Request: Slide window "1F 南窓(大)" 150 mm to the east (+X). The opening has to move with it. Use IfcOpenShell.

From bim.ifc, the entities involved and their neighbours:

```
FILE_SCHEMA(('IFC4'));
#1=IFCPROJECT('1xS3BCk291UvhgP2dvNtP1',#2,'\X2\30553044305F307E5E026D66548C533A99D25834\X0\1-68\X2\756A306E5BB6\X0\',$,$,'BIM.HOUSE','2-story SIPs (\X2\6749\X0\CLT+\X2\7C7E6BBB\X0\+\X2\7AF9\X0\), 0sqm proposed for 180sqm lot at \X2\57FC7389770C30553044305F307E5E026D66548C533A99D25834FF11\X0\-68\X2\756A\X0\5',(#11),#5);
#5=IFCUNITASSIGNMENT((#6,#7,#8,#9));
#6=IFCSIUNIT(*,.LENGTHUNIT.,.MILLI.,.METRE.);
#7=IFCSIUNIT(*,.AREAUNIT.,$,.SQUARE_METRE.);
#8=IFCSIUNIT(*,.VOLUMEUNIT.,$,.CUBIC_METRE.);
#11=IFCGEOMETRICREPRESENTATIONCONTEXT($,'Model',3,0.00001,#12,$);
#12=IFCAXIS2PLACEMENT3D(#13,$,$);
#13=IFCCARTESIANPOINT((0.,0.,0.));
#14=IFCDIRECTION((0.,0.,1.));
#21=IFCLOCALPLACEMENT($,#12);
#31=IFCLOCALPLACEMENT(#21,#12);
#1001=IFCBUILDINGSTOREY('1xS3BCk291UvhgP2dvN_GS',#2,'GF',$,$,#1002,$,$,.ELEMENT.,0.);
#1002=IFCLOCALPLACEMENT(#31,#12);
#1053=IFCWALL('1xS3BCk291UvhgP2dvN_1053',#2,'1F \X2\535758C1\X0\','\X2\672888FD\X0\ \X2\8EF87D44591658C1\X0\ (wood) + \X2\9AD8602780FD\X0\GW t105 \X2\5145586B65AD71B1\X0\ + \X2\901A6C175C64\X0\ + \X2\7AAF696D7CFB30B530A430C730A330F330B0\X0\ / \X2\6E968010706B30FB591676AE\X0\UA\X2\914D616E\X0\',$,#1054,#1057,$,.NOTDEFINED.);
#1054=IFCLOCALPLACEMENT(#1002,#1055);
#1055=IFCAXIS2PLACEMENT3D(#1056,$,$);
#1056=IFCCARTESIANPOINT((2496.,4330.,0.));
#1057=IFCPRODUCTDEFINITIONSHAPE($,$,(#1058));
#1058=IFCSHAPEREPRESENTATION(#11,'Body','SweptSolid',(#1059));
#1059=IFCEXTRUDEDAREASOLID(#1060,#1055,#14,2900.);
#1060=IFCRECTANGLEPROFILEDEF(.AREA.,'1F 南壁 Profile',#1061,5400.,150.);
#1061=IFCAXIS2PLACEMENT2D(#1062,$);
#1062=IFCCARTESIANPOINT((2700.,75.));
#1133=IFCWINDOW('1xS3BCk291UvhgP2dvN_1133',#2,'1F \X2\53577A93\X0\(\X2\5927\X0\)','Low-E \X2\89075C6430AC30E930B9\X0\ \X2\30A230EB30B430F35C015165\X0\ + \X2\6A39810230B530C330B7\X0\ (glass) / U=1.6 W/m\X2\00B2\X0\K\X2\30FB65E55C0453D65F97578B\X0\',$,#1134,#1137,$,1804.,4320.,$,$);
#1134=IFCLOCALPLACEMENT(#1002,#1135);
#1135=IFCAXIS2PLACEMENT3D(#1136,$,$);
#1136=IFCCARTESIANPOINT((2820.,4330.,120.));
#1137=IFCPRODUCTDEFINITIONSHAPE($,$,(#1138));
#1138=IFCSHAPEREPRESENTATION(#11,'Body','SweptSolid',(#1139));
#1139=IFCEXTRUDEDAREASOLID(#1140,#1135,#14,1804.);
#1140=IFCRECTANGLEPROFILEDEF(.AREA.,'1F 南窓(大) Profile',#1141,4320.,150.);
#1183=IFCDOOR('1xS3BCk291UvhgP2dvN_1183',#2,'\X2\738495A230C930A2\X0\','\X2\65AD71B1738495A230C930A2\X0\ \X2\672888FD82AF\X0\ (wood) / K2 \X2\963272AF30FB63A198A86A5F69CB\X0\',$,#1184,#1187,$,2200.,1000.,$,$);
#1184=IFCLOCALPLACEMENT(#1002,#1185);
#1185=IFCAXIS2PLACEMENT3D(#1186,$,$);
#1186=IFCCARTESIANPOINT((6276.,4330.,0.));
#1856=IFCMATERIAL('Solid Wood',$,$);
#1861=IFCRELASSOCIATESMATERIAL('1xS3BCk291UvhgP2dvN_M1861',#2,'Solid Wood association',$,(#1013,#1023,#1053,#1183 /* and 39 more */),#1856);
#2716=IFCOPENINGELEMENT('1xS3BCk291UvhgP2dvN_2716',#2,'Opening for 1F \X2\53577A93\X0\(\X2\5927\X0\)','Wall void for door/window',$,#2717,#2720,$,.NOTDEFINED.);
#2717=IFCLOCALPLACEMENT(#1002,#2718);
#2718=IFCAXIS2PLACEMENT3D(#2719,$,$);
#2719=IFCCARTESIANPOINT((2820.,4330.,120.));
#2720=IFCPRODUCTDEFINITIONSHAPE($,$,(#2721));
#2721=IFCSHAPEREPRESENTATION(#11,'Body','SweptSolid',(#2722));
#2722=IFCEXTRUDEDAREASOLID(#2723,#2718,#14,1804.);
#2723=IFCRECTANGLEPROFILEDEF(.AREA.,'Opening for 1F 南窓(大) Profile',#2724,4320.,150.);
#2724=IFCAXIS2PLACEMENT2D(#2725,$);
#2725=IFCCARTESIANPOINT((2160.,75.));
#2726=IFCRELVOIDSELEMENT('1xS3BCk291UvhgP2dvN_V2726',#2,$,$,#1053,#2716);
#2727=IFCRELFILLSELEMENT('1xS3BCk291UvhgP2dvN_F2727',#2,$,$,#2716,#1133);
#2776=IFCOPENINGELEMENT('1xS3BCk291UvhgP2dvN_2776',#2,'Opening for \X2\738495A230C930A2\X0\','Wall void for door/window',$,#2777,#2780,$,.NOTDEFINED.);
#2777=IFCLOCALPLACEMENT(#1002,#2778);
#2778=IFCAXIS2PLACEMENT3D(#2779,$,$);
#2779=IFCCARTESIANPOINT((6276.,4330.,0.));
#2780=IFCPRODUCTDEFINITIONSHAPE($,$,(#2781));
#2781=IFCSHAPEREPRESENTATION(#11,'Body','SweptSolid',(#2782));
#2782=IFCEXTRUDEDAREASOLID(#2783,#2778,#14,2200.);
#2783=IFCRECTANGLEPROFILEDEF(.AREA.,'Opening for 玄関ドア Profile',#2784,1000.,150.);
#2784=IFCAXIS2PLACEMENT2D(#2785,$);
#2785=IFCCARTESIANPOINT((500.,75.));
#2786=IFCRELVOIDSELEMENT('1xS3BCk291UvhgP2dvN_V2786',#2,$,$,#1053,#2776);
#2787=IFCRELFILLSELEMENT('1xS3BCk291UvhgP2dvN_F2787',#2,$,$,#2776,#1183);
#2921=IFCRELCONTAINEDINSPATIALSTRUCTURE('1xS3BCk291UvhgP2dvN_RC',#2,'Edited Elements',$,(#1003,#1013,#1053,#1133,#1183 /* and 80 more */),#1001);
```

```python
import ifcopenshell
import ifcopenshell.api.geometry
import ifcopenshell.util.placement
import ifcopenshell.util.unit

model = ifcopenshell.open("bim.ifc")
unit_scale = ifcopenshell.util.unit.calculate_unit_scale(model)

window = model.by_guid("1xS3BCk291UvhgP2dvN_1133")
opening = window.FillsVoids[0].RelatingOpeningElement
wall = opening.VoidsElements[0].RelatingBuildingElement

wall_matrix = ifcopenshell.util.placement.get_local_placement(wall.ObjectPlacement)
shift = wall_matrix[:3, 0] * 0.15 / unit_scale
before = ifcopenshell.util.placement.get_local_placement(window.ObjectPlacement)[:3, 3].copy()

# The window is not placed relative to its opening, so move both.
for product in (opening, window):
    matrix = ifcopenshell.util.placement.get_local_placement(product.ObjectPlacement)
    matrix[:3, 3] += shift
    ifcopenshell.api.geometry.edit_object_placement(model, product=product, matrix=matrix, is_si=False)

after = ifcopenshell.util.placement.get_local_placement(window.ObjectPlacement)[:3, 3]
print("window moved by", (after - before).round(3) + 0.0)

model.write("bim_edited.ifc")
```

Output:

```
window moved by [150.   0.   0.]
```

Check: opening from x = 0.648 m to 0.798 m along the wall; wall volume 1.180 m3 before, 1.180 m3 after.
